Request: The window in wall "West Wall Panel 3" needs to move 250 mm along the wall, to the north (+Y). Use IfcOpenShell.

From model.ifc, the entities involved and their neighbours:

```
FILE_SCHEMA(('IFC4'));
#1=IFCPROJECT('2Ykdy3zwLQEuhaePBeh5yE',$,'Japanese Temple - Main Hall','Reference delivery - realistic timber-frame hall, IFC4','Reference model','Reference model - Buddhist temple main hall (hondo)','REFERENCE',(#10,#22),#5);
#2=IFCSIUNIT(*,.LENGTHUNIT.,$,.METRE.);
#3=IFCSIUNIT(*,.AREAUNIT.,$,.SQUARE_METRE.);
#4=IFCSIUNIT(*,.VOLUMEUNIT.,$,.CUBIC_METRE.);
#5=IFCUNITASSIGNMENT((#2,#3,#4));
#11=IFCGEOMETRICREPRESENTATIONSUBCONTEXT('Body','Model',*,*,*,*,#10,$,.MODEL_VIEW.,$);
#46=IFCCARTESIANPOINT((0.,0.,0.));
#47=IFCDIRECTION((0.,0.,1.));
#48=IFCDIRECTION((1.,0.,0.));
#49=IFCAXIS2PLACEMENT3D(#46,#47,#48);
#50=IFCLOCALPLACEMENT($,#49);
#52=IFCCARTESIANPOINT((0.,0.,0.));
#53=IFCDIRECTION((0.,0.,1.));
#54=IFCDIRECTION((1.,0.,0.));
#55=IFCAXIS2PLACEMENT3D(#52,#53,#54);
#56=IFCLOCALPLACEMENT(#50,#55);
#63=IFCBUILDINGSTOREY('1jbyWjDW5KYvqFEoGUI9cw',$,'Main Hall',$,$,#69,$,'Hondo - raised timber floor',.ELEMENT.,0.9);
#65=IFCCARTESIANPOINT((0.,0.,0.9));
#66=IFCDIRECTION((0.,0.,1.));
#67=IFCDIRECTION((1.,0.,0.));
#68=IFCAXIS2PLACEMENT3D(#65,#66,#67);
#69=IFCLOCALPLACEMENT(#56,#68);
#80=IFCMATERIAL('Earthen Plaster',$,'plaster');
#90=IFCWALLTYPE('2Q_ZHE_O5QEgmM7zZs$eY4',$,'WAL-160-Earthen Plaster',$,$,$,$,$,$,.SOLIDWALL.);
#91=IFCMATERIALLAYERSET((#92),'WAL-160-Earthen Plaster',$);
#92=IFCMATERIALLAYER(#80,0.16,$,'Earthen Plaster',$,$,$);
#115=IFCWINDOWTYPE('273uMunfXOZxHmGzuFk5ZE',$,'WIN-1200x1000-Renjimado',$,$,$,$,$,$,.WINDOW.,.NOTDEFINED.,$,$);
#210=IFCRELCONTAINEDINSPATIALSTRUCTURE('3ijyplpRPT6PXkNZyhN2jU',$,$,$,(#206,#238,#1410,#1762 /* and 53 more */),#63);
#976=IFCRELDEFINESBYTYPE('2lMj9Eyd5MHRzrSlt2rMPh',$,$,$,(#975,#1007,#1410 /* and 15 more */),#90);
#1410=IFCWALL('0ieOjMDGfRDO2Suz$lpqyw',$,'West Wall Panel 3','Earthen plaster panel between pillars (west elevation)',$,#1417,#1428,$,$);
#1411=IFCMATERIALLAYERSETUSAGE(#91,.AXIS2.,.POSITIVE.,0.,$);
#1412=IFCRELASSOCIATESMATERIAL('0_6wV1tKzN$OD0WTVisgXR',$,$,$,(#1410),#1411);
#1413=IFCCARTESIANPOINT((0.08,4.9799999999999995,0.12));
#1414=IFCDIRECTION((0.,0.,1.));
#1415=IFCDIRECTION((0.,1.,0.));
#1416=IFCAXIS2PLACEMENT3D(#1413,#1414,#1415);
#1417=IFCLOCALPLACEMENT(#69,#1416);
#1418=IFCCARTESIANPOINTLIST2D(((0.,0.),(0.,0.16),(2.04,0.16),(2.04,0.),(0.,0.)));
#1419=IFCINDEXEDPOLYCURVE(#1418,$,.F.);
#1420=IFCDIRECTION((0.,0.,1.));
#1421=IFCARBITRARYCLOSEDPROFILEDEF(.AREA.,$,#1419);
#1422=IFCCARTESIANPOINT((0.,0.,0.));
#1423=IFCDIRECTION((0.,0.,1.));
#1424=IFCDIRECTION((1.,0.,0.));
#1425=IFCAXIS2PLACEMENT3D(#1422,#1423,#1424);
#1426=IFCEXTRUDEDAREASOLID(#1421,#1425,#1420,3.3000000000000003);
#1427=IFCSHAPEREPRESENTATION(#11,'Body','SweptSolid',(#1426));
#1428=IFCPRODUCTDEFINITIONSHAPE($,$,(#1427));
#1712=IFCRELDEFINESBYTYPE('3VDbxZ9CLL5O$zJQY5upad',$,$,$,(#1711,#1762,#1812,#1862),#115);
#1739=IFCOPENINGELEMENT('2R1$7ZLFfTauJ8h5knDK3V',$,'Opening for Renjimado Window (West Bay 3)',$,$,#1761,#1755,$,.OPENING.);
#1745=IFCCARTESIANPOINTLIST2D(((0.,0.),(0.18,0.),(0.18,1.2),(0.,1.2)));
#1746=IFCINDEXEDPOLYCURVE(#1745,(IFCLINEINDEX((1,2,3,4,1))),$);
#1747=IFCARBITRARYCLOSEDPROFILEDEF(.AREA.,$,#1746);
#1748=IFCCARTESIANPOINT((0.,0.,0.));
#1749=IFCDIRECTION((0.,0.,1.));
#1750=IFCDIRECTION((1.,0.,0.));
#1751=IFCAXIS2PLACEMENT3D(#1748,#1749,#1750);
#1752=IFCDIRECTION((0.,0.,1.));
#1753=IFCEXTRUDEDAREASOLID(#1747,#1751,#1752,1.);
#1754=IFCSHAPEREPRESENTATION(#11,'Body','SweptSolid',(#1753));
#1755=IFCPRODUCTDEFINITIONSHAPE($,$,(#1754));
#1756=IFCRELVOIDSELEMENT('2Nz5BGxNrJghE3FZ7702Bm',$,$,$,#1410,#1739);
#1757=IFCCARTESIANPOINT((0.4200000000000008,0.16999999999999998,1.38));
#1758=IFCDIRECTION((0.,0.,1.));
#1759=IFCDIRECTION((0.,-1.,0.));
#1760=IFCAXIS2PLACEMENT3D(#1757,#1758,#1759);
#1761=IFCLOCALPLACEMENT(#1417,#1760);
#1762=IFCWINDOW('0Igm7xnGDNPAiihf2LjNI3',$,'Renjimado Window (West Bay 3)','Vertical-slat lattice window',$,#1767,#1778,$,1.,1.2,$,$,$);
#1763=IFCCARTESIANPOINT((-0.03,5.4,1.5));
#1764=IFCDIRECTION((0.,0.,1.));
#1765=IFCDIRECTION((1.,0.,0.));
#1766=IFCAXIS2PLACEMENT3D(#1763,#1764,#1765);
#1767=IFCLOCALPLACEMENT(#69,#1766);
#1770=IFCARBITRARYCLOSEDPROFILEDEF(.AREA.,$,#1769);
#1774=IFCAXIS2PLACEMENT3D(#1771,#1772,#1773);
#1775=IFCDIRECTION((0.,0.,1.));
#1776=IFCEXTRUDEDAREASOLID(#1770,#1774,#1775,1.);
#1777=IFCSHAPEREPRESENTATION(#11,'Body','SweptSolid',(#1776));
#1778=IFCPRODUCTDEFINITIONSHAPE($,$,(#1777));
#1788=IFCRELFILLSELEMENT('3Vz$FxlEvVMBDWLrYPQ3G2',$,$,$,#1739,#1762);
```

```python
import ifcopenshell
import ifcopenshell.api.geometry
import ifcopenshell.util.placement

model = ifcopenshell.open("model.ifc")

window = model.by_guid("0Igm7xnGDNPAiihf2LjNI3")
opening = window.FillsVoids[0].RelatingOpeningElement
wall = opening.VoidsElements[0].RelatingBuildingElement

wall_matrix = ifcopenshell.util.placement.get_local_placement(wall.ObjectPlacement)
shift = wall_matrix[:3, 0] * 0.25
before = ifcopenshell.util.placement.get_local_placement(window.ObjectPlacement)[:3, 3].copy()

# The window is not placed relative to its opening, so move both.
for product in (opening, window):
    matrix = ifcopenshell.util.placement.get_local_placement(product.ObjectPlacement)
    matrix[:3, 3] += shift
    ifcopenshell.api.geometry.edit_object_placement(model, product=product, matrix=matrix, is_si=False)

after = ifcopenshell.util.placement.get_local_placement(window.ObjectPlacement)[:3, 3]
print("window moved by", (after - before).round(3) + 0.0)

model.write("model_updated.ifc")
```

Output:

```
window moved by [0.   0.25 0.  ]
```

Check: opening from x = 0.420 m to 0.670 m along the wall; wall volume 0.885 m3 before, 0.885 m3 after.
